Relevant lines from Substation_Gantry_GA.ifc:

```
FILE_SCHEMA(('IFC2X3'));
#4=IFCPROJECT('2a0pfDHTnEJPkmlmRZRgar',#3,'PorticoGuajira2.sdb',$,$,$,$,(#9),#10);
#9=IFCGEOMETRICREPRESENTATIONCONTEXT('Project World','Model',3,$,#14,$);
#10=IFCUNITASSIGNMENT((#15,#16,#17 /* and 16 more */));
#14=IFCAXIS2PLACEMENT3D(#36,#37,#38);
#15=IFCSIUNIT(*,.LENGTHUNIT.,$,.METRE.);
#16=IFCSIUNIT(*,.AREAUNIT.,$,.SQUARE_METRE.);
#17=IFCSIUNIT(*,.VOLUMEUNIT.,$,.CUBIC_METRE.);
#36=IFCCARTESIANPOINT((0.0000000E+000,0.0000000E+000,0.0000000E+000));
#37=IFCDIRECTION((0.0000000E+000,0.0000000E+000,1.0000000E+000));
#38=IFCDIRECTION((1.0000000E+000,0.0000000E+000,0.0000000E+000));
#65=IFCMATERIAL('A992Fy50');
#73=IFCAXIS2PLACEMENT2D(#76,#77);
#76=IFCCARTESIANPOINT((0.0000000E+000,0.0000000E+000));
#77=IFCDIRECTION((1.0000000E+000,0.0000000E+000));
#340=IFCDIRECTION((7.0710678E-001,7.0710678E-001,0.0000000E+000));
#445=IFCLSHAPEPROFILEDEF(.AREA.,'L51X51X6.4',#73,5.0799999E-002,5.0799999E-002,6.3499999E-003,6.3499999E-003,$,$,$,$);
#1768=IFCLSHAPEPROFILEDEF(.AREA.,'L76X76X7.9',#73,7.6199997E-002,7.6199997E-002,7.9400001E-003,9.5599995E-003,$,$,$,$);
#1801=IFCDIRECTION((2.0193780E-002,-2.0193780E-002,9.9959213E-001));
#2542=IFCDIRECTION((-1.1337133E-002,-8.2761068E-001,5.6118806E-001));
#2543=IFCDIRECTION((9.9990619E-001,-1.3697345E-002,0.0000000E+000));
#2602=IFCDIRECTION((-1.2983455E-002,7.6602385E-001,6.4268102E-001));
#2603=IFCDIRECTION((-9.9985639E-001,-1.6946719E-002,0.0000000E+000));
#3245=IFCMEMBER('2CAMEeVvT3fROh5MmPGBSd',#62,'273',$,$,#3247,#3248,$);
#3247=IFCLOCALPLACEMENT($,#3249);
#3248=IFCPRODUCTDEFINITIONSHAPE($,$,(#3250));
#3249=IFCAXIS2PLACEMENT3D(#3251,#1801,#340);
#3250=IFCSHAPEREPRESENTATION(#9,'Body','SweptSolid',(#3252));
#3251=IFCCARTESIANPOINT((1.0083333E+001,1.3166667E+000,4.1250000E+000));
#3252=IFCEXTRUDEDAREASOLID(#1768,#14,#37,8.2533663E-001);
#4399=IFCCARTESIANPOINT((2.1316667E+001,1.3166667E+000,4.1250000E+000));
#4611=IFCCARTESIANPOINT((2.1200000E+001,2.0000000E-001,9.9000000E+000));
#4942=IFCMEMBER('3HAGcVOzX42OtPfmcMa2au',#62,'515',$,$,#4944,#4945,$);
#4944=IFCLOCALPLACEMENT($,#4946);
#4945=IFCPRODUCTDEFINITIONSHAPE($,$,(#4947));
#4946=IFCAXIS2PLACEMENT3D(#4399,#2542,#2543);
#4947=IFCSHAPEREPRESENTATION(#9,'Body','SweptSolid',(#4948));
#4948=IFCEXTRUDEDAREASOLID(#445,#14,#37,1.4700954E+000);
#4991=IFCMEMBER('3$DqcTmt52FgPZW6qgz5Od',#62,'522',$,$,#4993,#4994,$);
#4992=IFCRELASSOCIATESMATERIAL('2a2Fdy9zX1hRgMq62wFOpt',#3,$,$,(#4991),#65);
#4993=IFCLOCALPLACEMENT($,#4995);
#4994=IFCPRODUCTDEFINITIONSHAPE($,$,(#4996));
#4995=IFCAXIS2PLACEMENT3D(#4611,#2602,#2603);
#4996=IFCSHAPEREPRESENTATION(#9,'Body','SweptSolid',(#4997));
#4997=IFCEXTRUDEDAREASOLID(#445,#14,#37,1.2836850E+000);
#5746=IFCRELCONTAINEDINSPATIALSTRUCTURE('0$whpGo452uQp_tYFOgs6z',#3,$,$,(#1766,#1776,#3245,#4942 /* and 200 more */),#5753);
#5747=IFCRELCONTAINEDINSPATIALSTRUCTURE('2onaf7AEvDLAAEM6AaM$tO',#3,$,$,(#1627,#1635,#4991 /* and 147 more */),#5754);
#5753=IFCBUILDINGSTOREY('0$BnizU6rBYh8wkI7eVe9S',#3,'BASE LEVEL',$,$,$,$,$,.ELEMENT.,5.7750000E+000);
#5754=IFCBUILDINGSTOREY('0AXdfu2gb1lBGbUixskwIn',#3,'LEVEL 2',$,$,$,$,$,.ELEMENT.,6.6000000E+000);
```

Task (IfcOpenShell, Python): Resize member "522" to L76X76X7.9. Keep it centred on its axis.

```python
import ifcopenshell
import ifcopenshell.util.element

model = ifcopenshell.open("Substation_Gantry_GA.ifc")

member = model.by_id(4991)
source = next(p for p in model.by_type("IfcLShapeProfileDef") if p.ProfileName == "L76X76X7.9")

body = next(r for r in member.Representation.Representations if r.RepresentationIdentifier == "Body")
solid = body.Items[0]
old_profile = solid.SweptArea

# Copy the section's sizes but keep this member's own profile position.
profile = ifcopenshell.util.element.copy(model, source)
profile.Position = old_profile.Position
solid.SweptArea = profile
if not model.get_total_inverses(old_profile):
    ifcopenshell.util.element.remove_deep2(model, old_profile)

print(solid.SweptArea)

model.write("Substation_Gantry_GA_rev.ifc")
```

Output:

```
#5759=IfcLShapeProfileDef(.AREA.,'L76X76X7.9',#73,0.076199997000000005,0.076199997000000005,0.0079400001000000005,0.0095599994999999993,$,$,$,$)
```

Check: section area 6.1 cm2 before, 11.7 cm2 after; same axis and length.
